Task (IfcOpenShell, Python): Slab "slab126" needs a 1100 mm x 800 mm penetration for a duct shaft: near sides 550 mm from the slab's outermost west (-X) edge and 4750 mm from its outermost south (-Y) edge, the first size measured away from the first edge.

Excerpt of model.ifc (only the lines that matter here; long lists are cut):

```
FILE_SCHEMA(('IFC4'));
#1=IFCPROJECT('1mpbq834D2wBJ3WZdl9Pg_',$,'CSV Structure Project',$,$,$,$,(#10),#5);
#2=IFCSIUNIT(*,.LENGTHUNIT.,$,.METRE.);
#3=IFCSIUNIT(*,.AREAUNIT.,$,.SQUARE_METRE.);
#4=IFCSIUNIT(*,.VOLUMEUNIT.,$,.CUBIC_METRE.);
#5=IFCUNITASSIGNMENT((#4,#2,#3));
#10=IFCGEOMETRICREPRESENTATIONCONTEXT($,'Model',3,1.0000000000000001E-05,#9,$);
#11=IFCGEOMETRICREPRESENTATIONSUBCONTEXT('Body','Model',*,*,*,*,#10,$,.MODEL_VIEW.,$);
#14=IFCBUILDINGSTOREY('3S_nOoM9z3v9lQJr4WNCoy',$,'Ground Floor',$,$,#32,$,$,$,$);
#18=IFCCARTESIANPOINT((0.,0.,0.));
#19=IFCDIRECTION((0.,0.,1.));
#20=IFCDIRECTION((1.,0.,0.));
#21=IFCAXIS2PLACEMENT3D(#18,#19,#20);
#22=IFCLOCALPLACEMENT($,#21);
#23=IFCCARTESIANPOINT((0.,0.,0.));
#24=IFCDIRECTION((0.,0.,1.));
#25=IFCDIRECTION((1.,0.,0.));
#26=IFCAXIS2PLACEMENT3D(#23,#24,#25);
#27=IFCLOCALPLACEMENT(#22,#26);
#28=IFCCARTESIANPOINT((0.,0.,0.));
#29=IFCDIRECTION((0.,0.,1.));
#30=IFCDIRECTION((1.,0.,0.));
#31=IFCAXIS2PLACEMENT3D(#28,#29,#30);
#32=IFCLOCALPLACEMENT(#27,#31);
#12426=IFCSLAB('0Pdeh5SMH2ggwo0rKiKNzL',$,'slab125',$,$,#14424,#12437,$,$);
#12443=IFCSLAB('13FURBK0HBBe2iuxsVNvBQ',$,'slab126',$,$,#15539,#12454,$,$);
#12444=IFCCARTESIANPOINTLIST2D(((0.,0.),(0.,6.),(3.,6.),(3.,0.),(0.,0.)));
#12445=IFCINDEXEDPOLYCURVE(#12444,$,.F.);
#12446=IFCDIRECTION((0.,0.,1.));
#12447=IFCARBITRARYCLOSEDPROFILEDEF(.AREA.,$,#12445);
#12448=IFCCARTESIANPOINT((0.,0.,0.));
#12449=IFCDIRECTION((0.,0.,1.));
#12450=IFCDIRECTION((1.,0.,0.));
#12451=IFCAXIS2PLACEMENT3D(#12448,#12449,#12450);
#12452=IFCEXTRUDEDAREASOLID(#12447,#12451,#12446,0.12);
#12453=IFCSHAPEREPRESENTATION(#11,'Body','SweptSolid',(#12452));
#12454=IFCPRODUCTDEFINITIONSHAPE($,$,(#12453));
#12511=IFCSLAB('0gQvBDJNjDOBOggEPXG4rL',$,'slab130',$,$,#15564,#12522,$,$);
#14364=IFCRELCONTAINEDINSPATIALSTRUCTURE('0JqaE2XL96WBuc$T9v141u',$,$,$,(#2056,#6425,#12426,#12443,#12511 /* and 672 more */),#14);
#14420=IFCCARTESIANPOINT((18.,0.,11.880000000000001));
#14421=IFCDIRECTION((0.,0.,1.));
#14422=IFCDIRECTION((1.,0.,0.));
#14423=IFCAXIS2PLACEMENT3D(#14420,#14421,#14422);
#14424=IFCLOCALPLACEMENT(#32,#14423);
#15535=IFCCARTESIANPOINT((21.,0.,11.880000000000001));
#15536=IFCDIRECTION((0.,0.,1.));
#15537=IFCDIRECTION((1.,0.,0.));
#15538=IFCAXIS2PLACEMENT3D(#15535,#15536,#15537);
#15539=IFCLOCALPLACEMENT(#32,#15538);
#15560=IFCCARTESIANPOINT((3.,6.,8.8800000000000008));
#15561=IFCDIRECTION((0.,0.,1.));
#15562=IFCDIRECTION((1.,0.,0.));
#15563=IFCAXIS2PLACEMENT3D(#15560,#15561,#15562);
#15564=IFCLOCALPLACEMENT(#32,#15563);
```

```python
import numpy as np
import ifcopenshell
import ifcopenshell.api.feature
import ifcopenshell.api.geometry
import ifcopenshell.api.root
import ifcopenshell.geom
import ifcopenshell.util.placement
import ifcopenshell.util.representation
import ifcopenshell.util.shape
import ifcopenshell.util.unit

model = ifcopenshell.open("model.ifc")
unit_scale = ifcopenshell.util.unit.calculate_unit_scale(model)
settings = ifcopenshell.geom.settings()


def volume(element):
    """Net volume in cubic metres, openings subtracted."""
    shape = ifcopenshell.geom.create_shape(settings, element)
    return ifcopenshell.util.shape.get_volume(shape.geometry)


slab = model.by_guid("13FURBK0HBBe2iuxsVNvBQ")
before = volume(slab)

# Extent in the slab's own axes, in metres. The edges named are its -X and -Y sides.
slab_shape = ifcopenshell.geom.create_shape(settings, slab)
vertices = ifcopenshell.util.shape.get_vertices(slab_shape.geometry)
x_min, y_min, bottom = vertices.min(axis=0)
top = vertices[:, 2].max()

opening = ifcopenshell.api.root.create_entity(model, ifc_class="IfcOpeningElement", name="Duct shaft opening", predefined_type="OPENING")
context = ifcopenshell.util.representation.get_context(model, "Model", "Body", "MODEL_VIEW")
width, depth = 1.1, 0.8
outline = [(0.0, 0.0), (width, 0.0), (width, depth), (0.0, depth), (0.0, 0.0)]
# Overshoot both faces by 50 mm so the cut is clean.
shape = ifcopenshell.api.geometry.add_slab_representation(
    model, context=context, depth=top - bottom + 0.1, polyline=outline
)
ifcopenshell.api.geometry.assign_representation(model, product=opening, representation=shape)

matrix = ifcopenshell.util.placement.get_local_placement(slab.ObjectPlacement)
matrix[:, 3] = matrix @ np.append(np.array([x_min + 0.55, y_min + 4.75, bottom - 0.05]) / unit_scale, 1.0)
ifcopenshell.api.geometry.edit_object_placement(model, product=opening, matrix=matrix, is_si=False)
ifcopenshell.api.feature.add_feature(model, feature=opening, element=slab)

after = volume(slab)

print(f"slab volume {before:.3f} -> {after:.3f} m3")

model.write("model_v2.ifc")
```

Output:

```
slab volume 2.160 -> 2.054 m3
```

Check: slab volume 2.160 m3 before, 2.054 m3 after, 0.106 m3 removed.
